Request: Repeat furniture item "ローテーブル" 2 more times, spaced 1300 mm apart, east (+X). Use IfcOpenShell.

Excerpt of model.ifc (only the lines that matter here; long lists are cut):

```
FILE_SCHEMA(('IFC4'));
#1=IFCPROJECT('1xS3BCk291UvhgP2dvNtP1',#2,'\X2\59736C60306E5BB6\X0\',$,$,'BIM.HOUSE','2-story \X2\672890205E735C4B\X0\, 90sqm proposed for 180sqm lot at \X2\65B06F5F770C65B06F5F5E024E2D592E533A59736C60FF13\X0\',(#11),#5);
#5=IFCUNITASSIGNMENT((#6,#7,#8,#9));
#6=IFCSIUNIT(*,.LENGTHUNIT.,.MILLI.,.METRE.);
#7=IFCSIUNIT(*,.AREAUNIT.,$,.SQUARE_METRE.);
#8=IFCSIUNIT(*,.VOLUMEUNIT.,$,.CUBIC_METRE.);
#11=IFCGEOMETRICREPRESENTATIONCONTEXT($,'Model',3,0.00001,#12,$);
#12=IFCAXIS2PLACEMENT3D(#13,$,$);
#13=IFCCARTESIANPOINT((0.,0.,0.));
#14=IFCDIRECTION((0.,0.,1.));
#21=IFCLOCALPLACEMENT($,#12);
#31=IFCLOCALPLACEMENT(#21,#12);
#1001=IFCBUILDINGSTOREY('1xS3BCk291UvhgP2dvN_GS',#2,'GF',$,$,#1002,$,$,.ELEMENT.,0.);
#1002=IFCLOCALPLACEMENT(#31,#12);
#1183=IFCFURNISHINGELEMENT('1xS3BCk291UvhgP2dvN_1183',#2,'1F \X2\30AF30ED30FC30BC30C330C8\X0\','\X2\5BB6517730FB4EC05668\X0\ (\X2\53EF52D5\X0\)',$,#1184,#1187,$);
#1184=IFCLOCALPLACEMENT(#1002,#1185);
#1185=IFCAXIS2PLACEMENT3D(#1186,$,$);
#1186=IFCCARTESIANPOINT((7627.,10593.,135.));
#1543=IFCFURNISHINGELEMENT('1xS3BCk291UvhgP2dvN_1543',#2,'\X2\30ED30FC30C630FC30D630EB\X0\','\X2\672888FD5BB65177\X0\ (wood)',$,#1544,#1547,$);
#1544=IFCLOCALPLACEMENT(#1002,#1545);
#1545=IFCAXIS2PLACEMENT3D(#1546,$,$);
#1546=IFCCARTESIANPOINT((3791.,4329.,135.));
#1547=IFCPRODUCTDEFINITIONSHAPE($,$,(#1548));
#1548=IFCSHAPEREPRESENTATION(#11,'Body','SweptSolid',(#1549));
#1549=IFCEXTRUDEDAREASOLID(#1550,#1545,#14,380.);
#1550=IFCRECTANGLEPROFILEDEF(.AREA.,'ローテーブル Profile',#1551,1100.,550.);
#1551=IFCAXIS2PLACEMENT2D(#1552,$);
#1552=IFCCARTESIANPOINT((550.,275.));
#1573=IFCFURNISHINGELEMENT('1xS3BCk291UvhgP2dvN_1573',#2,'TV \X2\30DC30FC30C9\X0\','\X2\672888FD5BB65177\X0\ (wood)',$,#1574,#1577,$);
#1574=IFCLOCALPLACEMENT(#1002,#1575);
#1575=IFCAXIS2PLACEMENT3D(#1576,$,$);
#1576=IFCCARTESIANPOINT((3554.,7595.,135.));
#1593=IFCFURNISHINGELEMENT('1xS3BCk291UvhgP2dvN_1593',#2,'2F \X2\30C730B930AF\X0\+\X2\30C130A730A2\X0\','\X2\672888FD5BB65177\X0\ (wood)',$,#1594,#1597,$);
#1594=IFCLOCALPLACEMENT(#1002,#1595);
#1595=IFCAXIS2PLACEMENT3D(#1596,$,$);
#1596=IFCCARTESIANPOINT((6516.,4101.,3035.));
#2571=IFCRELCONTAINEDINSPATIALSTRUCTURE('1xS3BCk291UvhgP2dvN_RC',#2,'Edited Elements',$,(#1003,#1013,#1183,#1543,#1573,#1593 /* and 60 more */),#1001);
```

```python
import numpy as np
import ifcopenshell
import ifcopenshell.api.geometry
import ifcopenshell.api.root
import ifcopenshell.util.element
import ifcopenshell.util.placement
import ifcopenshell.util.unit

model = ifcopenshell.open("model.ifc")
unit_scale = ifcopenshell.util.unit.calculate_unit_scale(model)


def reuse_history(source, copy):
    """copy_class also copies each property set's owner history, people and application; keep the originals."""
    for rel in copy.IsDefinedBy:
        if rel.is_a("IfcRelDefinesByProperties") and (history := rel.RelatingPropertyDefinition.OwnerHistory):
            rel.RelatingPropertyDefinition.OwnerHistory = source.OwnerHistory
            ifcopenshell.util.element.remove_deep2(model, history)


source = model.by_id(1543)
base = ifcopenshell.util.placement.get_local_placement(source.ObjectPlacement)
step = np.array([1.0, 0.0, 0.0]) * 1.3 / unit_scale

for i in range(1, 3):
    copy = ifcopenshell.api.root.copy_class(model, product=source)
    copy.Representation = ifcopenshell.util.element.copy_deep(
        model, source.Representation, exclude=["IfcGeometricRepresentationContext", "IfcRepresentationMap"]
    )
    reuse_history(source, copy)
    matrix = base.copy()
    matrix[:3, 3] += i * step
    print("added at", matrix[:3, 3].round(3) + 0.0)
    ifcopenshell.api.geometry.edit_object_placement(model, product=copy, matrix=matrix, is_si=False)

model.write("model_v2.ifc")
```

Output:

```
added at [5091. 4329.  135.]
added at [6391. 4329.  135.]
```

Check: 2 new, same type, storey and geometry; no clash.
